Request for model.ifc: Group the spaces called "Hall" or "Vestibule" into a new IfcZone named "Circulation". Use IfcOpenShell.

First a look at what the model holds.

```python
import ifcopenshell

model = ifcopenshell.open("model.ifc")
print(model.schema)
seen = {}
for space in model.by_type("IfcSpace"):
    seen[space.LongName] = seen.get(space.LongName, 0) + 1
for name, count in sorted(seen.items(), key=str):
    print(count, "x", name)
print("zones:", [z.Name for z in model.by_type("IfcZone")][:20])
```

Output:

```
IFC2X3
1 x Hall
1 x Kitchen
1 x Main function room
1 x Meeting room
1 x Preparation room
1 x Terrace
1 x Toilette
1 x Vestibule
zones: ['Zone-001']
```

```python
import ifcopenshell
import ifcopenshell.api.group
import ifcopenshell.api.root

model = ifcopenshell.open("model.ifc")

names = {"Hall", "Vestibule"}
spaces = [s for s in model.by_type("IfcSpace") if s.LongName in names]

zone = ifcopenshell.api.root.create_entity(model, ifc_class="IfcZone", name="Circulation")
ifcopenshell.api.group.assign_group(model, products=spaces, group=zone)
print(len(spaces), "spaces in", zone.Name)

model.write("model_v2.ifc")
```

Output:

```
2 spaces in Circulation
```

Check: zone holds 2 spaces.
